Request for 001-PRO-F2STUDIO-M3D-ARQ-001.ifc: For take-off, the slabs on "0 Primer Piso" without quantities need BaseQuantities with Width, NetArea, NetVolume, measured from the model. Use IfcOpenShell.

First a look at what the model holds.

```python
import ifcopenshell
import ifcopenshell.util.element
import ifcopenshell.util.unit

model = ifcopenshell.open("001-PRO-F2STUDIO-M3D-ARQ-001.ifc")
print(model.schema)
for unit_type in ("LENGTHUNIT", "AREAUNIT", "VOLUMEUNIT"):
    print(unit_type, ifcopenshell.util.unit.calculate_unit_scale(model, unit_type))
storey = next(s for s in model.by_type("IfcBuildingStorey") if s.Name == "0 Primer Piso")
slabs = [e for e in ifcopenshell.util.element.get_decomposition(storey) if e.is_a("IfcSlab")]
for e in sorted(slabs, key=lambda e: e.id()):
    print(e.id(), e.is_a(), e.Name, list(ifcopenshell.util.element.get_psets(e, qtos_only=True)), sep=" | ")
```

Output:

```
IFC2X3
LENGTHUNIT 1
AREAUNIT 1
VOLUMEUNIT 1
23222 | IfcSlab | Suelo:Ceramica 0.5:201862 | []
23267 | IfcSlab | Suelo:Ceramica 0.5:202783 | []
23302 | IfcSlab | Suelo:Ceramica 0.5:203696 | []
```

```python
import ifcopenshell
import ifcopenshell.api.pset
import ifcopenshell.geom
import ifcopenshell.util.element
import ifcopenshell.util.shape
import ifcopenshell.util.unit

model = ifcopenshell.open("001-PRO-F2STUDIO-M3D-ARQ-001.ifc")
unit_scale = ifcopenshell.util.unit.calculate_unit_scale(model)
area_scale = ifcopenshell.util.unit.calculate_unit_scale(model, "AREAUNIT")
volume_scale = ifcopenshell.util.unit.calculate_unit_scale(model, "VOLUMEUNIT")
settings = ifcopenshell.geom.settings()

storey = next(s for s in model.by_type("IfcBuildingStorey") if s.Name == "0 Primer Piso")
slabs = [e for e in ifcopenshell.util.element.get_decomposition(storey) if e.is_a("IfcSlab")]

for e in sorted(slabs, key=lambda e: e.id()):
    if ifcopenshell.util.element.get_psets(e, qtos_only=True, should_inherit=False):
        continue
    # Geometry comes back in metres, in the element's own axes.
    shape = ifcopenshell.geom.create_shape(settings, e)
    values = {
        "Width": ifcopenshell.util.shape.get_z(shape.geometry) / unit_scale,
        "NetArea": ifcopenshell.util.shape.get_footprint_area(shape.geometry) / area_scale,
        "NetVolume": ifcopenshell.util.shape.get_volume(shape.geometry) / volume_scale,
    }
    qto = ifcopenshell.api.pset.add_qto(model, product=e, name="BaseQuantities")
    ifcopenshell.api.pset.edit_qto(model, qto=qto, properties=values)
    print(e.id(), {k: round(v, 3) for k, v in values.items()})

model.write("001-PRO-F2STUDIO-M3D-ARQ-001_updated.ifc")
```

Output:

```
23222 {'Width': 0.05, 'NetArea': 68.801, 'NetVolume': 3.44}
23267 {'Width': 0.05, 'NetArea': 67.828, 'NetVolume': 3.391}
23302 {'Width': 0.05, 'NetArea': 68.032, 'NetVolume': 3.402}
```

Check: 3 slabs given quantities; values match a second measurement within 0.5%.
